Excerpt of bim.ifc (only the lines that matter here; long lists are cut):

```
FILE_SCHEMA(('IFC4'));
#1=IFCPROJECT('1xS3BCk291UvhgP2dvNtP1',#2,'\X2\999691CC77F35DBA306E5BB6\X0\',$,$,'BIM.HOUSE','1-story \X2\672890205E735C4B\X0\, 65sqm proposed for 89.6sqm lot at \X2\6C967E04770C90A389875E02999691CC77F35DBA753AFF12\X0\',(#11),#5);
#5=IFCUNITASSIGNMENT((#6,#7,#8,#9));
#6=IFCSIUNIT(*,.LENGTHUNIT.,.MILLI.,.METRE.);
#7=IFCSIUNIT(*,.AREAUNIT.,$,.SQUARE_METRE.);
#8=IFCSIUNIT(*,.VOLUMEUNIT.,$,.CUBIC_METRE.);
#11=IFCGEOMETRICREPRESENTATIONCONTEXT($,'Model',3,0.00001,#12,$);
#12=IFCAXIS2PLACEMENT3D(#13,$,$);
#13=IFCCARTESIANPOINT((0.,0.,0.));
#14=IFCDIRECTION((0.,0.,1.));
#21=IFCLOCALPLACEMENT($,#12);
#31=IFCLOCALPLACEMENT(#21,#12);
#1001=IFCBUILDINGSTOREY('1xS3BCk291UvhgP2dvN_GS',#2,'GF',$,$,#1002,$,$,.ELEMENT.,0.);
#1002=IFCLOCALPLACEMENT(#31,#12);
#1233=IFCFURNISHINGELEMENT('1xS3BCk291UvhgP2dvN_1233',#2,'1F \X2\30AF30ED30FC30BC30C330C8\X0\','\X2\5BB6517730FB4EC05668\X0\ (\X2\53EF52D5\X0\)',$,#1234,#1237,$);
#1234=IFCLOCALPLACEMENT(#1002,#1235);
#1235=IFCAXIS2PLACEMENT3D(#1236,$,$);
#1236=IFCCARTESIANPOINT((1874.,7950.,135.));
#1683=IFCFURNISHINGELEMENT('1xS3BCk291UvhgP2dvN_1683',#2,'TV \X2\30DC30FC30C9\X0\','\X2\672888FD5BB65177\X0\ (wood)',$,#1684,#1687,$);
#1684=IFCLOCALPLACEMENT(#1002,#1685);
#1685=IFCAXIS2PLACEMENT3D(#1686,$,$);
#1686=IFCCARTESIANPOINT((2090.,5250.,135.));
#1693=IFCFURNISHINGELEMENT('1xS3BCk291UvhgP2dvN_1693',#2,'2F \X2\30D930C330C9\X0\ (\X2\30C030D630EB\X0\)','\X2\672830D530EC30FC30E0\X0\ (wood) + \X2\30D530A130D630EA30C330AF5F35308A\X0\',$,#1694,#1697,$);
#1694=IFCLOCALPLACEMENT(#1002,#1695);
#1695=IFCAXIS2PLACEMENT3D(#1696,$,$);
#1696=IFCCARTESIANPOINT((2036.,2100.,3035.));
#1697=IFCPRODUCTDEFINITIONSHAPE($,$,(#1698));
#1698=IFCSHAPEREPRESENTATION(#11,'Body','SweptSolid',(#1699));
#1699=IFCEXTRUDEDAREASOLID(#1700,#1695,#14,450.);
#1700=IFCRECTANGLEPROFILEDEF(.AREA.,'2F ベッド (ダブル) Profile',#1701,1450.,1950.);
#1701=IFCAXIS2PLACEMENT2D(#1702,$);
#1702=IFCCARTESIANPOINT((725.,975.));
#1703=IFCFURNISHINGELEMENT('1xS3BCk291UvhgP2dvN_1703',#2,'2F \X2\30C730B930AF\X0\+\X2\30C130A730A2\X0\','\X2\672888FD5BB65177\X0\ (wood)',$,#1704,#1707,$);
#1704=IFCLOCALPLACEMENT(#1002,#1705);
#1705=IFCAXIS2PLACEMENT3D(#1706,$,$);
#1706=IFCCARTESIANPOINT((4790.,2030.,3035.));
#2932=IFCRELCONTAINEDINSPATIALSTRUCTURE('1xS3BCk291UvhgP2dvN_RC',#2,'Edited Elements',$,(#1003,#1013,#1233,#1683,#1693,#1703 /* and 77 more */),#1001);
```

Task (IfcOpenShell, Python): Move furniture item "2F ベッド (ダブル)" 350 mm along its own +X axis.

```python
import ifcopenshell
import ifcopenshell.api.geometry
import ifcopenshell.util.placement

model = ifcopenshell.open("bim.ifc")

item = model.by_guid("1xS3BCk291UvhgP2dvN_1693")
matrix = ifcopenshell.util.placement.get_local_placement(item.ObjectPlacement)
matrix[:3, 3] += matrix[:3, 0] * 350.0
ifcopenshell.api.geometry.edit_object_placement(model, product=item, matrix=matrix, is_si=False)

print(ifcopenshell.util.placement.get_local_placement(item.ObjectPlacement).round(3) + 0.0)

model.write("bim-out.ifc")
```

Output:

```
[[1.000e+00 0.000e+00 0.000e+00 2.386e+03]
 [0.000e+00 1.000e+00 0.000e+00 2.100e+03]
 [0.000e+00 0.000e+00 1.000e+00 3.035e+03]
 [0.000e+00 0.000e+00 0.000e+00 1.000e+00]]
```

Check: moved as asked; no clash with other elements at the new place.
